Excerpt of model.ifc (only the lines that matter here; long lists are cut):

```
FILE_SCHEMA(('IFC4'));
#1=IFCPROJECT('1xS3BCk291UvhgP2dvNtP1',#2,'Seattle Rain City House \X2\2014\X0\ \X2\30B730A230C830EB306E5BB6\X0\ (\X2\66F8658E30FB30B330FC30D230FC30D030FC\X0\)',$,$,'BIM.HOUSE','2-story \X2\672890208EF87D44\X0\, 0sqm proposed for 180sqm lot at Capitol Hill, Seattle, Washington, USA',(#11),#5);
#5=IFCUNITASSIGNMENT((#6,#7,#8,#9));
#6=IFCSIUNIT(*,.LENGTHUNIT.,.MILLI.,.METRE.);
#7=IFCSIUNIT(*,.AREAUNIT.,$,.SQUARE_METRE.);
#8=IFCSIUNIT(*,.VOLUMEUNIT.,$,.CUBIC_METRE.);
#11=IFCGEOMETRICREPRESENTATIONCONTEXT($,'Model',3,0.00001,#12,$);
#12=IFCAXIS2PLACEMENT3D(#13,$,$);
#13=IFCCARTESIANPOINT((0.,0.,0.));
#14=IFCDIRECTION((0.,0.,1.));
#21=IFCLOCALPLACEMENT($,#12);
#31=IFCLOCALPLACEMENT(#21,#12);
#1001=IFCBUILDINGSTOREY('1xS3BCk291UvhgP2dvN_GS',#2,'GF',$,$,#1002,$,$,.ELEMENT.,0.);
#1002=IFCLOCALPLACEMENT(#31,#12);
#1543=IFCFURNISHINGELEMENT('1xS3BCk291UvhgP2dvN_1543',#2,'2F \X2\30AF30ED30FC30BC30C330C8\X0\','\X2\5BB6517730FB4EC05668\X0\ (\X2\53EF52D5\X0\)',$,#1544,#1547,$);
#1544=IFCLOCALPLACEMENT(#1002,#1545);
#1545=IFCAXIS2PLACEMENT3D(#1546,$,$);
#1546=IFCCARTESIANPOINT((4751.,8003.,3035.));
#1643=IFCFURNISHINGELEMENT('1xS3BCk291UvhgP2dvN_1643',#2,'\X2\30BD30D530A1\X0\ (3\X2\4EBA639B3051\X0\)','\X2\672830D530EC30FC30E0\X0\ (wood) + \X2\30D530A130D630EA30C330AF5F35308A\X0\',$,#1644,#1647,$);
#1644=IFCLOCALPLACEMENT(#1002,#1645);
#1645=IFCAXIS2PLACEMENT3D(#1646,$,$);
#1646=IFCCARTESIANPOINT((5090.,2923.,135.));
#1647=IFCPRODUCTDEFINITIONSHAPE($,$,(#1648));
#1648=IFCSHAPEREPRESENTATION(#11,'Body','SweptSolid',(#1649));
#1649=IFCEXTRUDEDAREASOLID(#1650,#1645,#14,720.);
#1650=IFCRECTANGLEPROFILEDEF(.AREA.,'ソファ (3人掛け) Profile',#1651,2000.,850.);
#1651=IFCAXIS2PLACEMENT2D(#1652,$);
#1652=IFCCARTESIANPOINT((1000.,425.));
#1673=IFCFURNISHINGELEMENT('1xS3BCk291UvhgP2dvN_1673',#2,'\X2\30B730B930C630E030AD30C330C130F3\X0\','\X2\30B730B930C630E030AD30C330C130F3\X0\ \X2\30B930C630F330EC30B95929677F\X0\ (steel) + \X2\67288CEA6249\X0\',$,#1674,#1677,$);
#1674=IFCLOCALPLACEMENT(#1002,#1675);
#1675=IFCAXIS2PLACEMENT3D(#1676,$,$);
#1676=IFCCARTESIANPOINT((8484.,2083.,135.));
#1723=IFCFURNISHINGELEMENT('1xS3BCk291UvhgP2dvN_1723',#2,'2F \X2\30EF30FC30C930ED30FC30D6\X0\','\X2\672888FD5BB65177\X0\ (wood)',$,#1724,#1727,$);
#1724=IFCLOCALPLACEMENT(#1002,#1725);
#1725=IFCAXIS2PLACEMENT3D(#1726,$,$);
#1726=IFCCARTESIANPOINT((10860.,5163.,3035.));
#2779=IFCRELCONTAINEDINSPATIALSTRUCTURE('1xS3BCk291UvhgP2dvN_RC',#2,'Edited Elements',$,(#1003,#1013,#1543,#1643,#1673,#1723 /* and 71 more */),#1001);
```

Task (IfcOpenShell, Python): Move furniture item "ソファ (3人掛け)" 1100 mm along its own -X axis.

```python
import ifcopenshell
import ifcopenshell.api.geometry
import ifcopenshell.util.placement

model = ifcopenshell.open("model.ifc")

item = model.by_id(1643)
matrix = ifcopenshell.util.placement.get_local_placement(item.ObjectPlacement)
matrix[:3, 3] -= matrix[:3, 0] * 1100.0
ifcopenshell.api.geometry.edit_object_placement(model, product=item, matrix=matrix, is_si=False)

print(ifcopenshell.util.placement.get_local_placement(item.ObjectPlacement).round(3) + 0.0)

model.write("model_rev.ifc")
```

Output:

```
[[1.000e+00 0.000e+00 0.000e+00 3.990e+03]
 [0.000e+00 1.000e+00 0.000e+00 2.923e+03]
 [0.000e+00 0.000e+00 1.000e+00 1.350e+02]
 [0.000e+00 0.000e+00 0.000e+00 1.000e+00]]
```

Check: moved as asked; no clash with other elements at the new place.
